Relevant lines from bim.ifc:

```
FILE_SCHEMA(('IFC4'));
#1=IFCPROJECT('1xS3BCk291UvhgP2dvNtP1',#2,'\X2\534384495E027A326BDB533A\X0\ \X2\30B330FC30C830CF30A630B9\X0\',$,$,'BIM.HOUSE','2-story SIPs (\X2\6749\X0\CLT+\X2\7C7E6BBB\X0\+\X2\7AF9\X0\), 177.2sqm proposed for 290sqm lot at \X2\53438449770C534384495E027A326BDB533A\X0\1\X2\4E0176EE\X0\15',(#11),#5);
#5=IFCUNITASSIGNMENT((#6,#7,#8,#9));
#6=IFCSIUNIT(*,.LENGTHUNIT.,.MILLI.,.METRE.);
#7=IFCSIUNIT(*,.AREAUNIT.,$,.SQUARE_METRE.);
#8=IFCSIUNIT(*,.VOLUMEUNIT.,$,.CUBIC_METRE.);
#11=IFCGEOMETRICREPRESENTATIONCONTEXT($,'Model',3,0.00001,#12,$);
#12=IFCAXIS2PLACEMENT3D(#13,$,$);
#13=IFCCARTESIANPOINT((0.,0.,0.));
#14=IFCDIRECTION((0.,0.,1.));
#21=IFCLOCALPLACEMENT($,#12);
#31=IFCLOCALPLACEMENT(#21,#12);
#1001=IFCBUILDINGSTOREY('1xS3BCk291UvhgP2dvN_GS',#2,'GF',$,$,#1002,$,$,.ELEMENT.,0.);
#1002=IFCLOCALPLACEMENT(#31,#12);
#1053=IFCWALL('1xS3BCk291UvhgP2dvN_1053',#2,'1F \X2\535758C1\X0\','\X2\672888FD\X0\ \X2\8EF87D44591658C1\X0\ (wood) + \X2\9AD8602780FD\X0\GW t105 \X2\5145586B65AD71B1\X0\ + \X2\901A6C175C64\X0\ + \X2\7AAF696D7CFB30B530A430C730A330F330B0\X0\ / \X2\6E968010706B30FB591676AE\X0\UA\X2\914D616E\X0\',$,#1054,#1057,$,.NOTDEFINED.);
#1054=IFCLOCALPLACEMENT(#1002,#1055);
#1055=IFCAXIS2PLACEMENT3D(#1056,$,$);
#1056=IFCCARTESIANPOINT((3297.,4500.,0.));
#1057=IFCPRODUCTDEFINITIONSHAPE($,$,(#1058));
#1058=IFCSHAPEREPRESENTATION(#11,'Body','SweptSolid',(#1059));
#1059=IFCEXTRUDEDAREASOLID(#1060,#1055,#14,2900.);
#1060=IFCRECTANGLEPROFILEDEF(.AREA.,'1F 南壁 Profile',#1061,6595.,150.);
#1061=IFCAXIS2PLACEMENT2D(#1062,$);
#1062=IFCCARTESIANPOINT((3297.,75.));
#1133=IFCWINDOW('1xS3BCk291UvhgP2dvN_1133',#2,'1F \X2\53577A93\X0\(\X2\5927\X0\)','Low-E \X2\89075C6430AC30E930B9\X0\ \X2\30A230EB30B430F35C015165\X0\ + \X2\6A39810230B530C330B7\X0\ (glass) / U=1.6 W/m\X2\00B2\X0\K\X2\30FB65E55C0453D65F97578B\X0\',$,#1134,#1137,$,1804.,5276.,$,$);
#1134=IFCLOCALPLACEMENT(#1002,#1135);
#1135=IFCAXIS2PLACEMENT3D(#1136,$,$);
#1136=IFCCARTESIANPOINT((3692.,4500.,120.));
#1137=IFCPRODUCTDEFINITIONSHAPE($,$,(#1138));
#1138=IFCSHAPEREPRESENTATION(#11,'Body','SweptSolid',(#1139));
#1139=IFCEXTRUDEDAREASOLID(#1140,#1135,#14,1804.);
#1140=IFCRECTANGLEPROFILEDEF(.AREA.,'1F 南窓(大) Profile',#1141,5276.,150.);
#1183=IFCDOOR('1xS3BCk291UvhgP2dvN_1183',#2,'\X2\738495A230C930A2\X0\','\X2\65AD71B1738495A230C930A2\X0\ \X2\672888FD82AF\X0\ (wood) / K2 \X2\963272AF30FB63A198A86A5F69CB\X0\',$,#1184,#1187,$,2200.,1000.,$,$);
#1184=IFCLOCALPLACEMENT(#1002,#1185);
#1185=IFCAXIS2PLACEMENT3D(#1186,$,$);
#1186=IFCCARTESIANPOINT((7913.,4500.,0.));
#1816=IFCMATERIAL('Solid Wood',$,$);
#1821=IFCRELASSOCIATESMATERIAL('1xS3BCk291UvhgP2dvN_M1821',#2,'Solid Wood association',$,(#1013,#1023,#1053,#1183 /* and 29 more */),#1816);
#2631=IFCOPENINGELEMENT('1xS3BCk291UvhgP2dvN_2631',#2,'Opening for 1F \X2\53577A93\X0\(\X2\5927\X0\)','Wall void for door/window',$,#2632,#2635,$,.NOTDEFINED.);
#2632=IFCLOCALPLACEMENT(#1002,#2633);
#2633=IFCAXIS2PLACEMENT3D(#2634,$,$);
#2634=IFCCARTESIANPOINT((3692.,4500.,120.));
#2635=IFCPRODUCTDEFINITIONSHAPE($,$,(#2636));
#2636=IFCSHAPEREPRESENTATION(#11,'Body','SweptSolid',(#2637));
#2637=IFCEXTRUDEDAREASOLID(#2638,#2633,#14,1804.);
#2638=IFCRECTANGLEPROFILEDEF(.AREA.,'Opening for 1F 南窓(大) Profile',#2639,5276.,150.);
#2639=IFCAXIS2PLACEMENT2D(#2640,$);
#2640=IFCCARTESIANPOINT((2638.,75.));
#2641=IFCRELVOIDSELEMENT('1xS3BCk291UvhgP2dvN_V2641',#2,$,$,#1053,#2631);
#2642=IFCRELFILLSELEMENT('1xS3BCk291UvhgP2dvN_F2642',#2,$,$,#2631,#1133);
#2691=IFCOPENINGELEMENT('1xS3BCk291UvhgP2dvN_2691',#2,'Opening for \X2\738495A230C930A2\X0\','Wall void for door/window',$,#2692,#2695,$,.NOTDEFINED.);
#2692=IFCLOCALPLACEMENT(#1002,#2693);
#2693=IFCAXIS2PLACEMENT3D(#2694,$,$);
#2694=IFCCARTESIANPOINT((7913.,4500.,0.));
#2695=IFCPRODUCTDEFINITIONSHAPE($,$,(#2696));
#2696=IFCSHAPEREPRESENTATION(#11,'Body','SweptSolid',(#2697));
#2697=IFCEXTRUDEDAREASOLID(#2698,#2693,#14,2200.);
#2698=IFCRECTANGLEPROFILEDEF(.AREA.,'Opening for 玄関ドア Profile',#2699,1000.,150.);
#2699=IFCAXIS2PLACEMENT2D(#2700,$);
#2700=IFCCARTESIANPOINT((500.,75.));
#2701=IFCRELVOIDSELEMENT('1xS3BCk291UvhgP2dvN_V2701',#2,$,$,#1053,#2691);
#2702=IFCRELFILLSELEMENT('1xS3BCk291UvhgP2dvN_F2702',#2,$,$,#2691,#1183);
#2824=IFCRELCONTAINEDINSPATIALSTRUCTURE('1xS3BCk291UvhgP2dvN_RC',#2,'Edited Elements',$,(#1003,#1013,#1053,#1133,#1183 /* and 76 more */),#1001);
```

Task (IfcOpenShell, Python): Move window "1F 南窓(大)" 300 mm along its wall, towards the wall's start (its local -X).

```python
import ifcopenshell
import ifcopenshell.api.geometry
import ifcopenshell.util.placement
import ifcopenshell.util.unit

model = ifcopenshell.open("bim.ifc")
unit_scale = ifcopenshell.util.unit.calculate_unit_scale(model)

window = model.by_guid("1xS3BCk291UvhgP2dvN_1133")
opening = window.FillsVoids[0].RelatingOpeningElement
wall = opening.VoidsElements[0].RelatingBuildingElement

wall_matrix = ifcopenshell.util.placement.get_local_placement(wall.ObjectPlacement)
shift = wall_matrix[:3, 0] * -0.3 / unit_scale
before = ifcopenshell.util.placement.get_local_placement(window.ObjectPlacement)[:3, 3].copy()

# The window is not placed relative to its opening, so move both.
for product in (opening, window):
    matrix = ifcopenshell.util.placement.get_local_placement(product.ObjectPlacement)
    matrix[:3, 3] += shift
    ifcopenshell.api.geometry.edit_object_placement(model, product=product, matrix=matrix, is_si=False)

after = ifcopenshell.util.placement.get_local_placement(window.ObjectPlacement)[:3, 3]
print("window moved by", (after - before).round(3) + 0.0)

model.write("bim-out.ifc")
```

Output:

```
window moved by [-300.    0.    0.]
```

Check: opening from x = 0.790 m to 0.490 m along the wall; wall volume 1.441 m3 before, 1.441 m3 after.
